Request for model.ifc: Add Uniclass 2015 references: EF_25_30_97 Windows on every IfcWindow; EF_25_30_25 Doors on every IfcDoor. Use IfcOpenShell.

First a look at what the model holds.

```python
import ifcopenshell

model = ifcopenshell.open("model.ifc")
print(model.schema)
print("classifications:", [c.Name for c in model.by_type("IfcClassification")])
for ifc_class in ("IfcDoor", "IfcRoof", "IfcStair", "IfcWall", "IfcWindow"):
    print(ifc_class, len(model.by_type(ifc_class)))
```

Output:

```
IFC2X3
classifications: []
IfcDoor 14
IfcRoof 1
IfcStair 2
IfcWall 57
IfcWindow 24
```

```python
import ifcopenshell
import ifcopenshell.api.classification

model = ifcopenshell.open("model.ifc")

# IFC2X3 requires Source and Edition and has no link from the project to the system.
system = model.create_entity("IfcClassification", Source="NBS", Edition="2015", Name="Uniclass 2015")

codes = {
    "IfcWindow": ("EF_25_30_97", "Windows"),
    "IfcDoor": ("EF_25_30_25", "Doors"),
}
for ifc_class, (code, name) in codes.items():
    products = model.by_type(ifc_class)
    ifcopenshell.api.classification.add_reference(
        model, products=products, classification=system, identification=code, name=name
    )
    print(code, len(products))

model.write("model_rev.ifc")
```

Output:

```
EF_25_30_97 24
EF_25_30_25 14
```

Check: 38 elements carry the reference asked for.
